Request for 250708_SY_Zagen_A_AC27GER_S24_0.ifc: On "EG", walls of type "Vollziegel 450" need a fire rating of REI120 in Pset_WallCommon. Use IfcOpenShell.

First a look at what the model holds.

```python
import ifcopenshell
import ifcopenshell.util.element

model = ifcopenshell.open("250708_SY_Zagen_A_AC27GER_S24_0.ifc")
print(model.schema)
storey = next(s for s in model.by_type("IfcBuildingStorey") if s.Name == "EG")
walls = [e for e in ifcopenshell.util.element.get_decomposition(storey) if e.is_a("IfcWall")]
seen = {}
for e in walls:
    element_type = ifcopenshell.util.element.get_type(e)
    key = (element_type.Name if element_type != e and element_type else None, ifcopenshell.util.element.get_pset(e, "Pset_WallCommon", "FireRating"))
    seen[key] = seen.get(key, 0) + 1
for (name, value), count in sorted(seen.items(), key=str):
    print(count, "x", name, "|", value)
```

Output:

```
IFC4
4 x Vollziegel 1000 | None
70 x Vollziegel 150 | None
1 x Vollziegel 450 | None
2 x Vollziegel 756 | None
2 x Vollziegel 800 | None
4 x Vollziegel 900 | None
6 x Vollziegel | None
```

```python
import ifcopenshell
import ifcopenshell.api.pset
import ifcopenshell.util.element

model = ifcopenshell.open("250708_SY_Zagen_A_AC27GER_S24_0.ifc")

storey = next(s for s in model.by_type("IfcBuildingStorey") if s.Name == "EG")
walls = [e for e in ifcopenshell.util.element.get_decomposition(storey) if e.is_a("IfcWall")]

count = 0
for e in walls:
    element_type = ifcopenshell.util.element.get_type(e)
    if element_type in (None, e) or element_type.Name != "Vollziegel 450":
        continue
    # add_pset returns the element's existing set when there is one.
    pset = ifcopenshell.api.pset.add_pset(model, product=e, name="Pset_WallCommon")
    ifcopenshell.api.pset.edit_pset(model, pset=pset, properties={"FireRating": "REI120"})
    count += 1

print(count, "walls updated")

model.write("250708_SY_Zagen_A_AC27GER_S24_0-out.ifc")
```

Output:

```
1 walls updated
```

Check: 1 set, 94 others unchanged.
